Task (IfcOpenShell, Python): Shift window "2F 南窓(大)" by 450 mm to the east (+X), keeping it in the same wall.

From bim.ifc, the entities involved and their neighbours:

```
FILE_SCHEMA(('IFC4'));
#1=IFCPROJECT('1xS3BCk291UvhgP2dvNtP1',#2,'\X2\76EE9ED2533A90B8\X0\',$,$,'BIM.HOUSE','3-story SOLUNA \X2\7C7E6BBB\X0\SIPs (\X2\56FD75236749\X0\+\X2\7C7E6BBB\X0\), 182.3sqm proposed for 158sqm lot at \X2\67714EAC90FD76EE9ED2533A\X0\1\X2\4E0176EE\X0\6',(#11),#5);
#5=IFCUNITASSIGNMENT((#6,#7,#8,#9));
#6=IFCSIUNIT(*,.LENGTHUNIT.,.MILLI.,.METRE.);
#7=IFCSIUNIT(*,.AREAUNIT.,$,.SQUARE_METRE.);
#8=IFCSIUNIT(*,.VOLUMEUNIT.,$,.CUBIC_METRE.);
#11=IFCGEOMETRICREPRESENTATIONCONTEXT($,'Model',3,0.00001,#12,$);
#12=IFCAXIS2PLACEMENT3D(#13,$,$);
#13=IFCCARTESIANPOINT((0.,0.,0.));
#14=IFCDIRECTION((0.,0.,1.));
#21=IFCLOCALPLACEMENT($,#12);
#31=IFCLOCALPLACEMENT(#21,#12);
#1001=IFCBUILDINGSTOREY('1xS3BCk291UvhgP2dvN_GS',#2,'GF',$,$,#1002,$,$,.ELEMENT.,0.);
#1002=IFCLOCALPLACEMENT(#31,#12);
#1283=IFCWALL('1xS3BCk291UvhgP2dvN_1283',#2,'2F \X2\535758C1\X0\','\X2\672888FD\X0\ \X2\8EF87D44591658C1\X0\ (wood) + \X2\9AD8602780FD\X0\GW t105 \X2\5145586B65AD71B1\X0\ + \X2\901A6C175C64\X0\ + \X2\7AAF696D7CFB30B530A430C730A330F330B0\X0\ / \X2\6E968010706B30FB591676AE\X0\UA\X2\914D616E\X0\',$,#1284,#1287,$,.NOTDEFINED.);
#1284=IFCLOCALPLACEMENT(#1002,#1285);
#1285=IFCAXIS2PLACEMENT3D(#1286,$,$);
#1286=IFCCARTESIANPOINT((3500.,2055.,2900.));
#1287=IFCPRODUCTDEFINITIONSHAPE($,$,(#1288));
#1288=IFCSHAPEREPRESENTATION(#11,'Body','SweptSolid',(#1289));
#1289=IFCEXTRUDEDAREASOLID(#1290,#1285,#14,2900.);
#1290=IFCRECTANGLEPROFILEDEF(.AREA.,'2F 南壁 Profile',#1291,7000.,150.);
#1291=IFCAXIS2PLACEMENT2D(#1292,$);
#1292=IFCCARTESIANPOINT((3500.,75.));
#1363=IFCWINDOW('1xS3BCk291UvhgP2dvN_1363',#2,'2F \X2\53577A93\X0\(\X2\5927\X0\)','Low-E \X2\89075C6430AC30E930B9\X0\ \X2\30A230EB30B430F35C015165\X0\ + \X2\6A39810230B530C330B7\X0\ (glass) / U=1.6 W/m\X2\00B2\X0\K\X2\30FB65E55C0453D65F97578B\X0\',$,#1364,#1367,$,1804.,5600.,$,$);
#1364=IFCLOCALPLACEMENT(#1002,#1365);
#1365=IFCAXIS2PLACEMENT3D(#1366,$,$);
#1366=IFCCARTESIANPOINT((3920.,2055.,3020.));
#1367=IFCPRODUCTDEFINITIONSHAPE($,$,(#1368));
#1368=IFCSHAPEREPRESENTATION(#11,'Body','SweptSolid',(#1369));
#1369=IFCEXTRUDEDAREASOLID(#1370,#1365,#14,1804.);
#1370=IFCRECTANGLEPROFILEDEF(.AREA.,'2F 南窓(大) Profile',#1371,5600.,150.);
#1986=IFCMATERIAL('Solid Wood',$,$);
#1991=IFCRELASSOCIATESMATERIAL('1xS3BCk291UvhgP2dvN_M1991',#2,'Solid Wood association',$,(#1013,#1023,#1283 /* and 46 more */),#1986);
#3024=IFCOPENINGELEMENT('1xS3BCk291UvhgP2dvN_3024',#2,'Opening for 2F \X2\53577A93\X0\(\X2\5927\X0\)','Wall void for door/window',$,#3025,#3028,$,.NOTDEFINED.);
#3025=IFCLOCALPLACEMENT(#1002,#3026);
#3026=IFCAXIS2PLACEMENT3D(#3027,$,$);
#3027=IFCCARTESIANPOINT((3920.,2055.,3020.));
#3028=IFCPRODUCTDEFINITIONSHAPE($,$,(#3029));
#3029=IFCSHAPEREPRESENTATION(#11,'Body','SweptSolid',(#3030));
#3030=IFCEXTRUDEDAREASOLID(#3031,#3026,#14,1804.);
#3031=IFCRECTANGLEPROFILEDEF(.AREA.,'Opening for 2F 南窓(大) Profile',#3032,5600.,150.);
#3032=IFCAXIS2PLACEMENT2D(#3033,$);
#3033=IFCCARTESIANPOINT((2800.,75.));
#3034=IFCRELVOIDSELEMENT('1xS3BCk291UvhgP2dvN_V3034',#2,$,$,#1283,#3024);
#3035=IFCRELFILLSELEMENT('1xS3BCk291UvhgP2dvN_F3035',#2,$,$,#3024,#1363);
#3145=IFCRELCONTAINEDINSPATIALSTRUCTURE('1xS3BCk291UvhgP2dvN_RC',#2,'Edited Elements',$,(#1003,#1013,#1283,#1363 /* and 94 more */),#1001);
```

```python
import ifcopenshell
import ifcopenshell.api.geometry
import ifcopenshell.util.placement
import ifcopenshell.util.unit

model = ifcopenshell.open("bim.ifc")
unit_scale = ifcopenshell.util.unit.calculate_unit_scale(model)

window = model.by_guid("1xS3BCk291UvhgP2dvN_1363")
opening = window.FillsVoids[0].RelatingOpeningElement
wall = opening.VoidsElements[0].RelatingBuildingElement

wall_matrix = ifcopenshell.util.placement.get_local_placement(wall.ObjectPlacement)
shift = wall_matrix[:3, 0] * 0.45 / unit_scale
before = ifcopenshell.util.placement.get_local_placement(window.ObjectPlacement)[:3, 3].copy()

# The window is not placed relative to its opening, so move both.
for product in (opening, window):
    matrix = ifcopenshell.util.placement.get_local_placement(product.ObjectPlacement)
    matrix[:3, 3] += shift
    ifcopenshell.api.geometry.edit_object_placement(model, product=product, matrix=matrix, is_si=False)

after = ifcopenshell.util.placement.get_local_placement(window.ObjectPlacement)[:3, 3]
print("window moved by", (after - before).round(3) + 0.0)

model.write("bim_edited.ifc")
```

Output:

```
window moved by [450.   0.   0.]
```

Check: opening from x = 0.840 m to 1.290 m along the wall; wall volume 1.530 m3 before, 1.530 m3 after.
